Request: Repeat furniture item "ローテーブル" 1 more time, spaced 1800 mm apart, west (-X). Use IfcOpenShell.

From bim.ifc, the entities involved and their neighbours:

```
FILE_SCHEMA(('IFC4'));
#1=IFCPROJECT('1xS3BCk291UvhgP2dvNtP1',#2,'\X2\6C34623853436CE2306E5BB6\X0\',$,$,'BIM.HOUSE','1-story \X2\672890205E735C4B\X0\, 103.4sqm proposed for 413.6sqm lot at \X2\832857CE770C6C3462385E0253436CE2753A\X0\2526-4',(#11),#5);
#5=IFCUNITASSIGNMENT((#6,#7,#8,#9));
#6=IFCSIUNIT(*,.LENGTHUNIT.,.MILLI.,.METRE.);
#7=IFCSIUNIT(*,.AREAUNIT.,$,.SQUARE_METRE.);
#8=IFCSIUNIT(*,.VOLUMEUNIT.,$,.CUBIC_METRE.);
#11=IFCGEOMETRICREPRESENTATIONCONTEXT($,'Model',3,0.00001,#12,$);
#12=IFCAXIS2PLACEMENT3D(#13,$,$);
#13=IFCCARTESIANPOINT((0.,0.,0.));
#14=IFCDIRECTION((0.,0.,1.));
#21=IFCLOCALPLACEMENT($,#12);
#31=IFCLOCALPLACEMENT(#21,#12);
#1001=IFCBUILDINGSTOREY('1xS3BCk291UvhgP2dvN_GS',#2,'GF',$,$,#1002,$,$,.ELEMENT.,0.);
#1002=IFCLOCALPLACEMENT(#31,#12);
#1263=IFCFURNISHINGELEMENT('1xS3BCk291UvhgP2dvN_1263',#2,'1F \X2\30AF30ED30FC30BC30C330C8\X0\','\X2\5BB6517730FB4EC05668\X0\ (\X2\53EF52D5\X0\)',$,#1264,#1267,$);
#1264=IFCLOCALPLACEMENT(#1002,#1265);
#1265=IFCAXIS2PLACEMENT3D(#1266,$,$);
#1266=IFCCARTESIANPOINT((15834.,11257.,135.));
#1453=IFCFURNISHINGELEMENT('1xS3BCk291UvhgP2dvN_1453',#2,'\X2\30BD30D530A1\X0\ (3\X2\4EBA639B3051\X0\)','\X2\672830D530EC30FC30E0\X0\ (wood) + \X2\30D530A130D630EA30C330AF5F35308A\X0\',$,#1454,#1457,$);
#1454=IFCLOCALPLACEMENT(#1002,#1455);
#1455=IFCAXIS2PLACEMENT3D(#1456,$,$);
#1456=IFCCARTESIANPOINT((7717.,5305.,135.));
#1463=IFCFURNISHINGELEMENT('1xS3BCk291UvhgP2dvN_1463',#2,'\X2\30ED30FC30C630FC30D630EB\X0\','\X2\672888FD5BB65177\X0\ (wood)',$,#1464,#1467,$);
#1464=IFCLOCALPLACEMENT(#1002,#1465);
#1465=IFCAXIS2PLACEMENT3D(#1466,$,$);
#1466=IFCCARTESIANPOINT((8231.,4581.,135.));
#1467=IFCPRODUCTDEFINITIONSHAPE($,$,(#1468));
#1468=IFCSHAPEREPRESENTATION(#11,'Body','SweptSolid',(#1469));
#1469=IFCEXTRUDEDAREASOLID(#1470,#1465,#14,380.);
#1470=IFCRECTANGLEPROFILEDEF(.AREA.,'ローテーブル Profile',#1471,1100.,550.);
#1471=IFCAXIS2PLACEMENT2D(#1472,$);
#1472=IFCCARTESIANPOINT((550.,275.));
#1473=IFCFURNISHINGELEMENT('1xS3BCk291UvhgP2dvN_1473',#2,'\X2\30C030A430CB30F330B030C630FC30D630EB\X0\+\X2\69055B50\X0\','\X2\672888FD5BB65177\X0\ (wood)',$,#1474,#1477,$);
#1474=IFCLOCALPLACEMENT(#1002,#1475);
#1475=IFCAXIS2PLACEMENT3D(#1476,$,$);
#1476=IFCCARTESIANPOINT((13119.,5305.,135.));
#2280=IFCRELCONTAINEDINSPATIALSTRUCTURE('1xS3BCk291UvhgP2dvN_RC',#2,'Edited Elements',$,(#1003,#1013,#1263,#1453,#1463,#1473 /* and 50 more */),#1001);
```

```python
import numpy as np
import ifcopenshell
import ifcopenshell.api.geometry
import ifcopenshell.api.root
import ifcopenshell.util.element
import ifcopenshell.util.placement
import ifcopenshell.util.unit

model = ifcopenshell.open("bim.ifc")
unit_scale = ifcopenshell.util.unit.calculate_unit_scale(model)


def reuse_history(source, copy):
    """copy_class also copies each property set's owner history, people and application; keep the originals."""
    for rel in copy.IsDefinedBy:
        if rel.is_a("IfcRelDefinesByProperties") and (history := rel.RelatingPropertyDefinition.OwnerHistory):
            rel.RelatingPropertyDefinition.OwnerHistory = source.OwnerHistory
            ifcopenshell.util.element.remove_deep2(model, history)


source = model.by_id(1463)
base = ifcopenshell.util.placement.get_local_placement(source.ObjectPlacement)
step = np.array([-1.0, 0.0, 0.0]) * 1.8 / unit_scale

for i in range(1, 2):
    copy = ifcopenshell.api.root.copy_class(model, product=source)
    copy.Representation = ifcopenshell.util.element.copy_deep(
        model, source.Representation, exclude=["IfcGeometricRepresentationContext", "IfcRepresentationMap"]
    )
    reuse_history(source, copy)
    matrix = base.copy()
    matrix[:3, 3] += i * step
    print("added at", matrix[:3, 3].round(3) + 0.0)
    ifcopenshell.api.geometry.edit_object_placement(model, product=copy, matrix=matrix, is_si=False)

model.write("bim-out.ifc")
```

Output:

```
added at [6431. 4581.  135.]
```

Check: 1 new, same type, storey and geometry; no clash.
